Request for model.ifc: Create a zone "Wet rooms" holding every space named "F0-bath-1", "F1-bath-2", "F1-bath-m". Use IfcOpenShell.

First a look at what the model holds.

```python
import ifcopenshell

model = ifcopenshell.open("model.ifc")
print(model.schema)
seen = {}
for space in model.by_type("IfcSpace"):
    seen[space.LongName] = seen.get(space.LongName, 0) + 1
for name, count in sorted(seen.items(), key=str):
    print(count, "x", name)
print("zones:", [z.Name for z in model.by_type("IfcZone")][:20])
```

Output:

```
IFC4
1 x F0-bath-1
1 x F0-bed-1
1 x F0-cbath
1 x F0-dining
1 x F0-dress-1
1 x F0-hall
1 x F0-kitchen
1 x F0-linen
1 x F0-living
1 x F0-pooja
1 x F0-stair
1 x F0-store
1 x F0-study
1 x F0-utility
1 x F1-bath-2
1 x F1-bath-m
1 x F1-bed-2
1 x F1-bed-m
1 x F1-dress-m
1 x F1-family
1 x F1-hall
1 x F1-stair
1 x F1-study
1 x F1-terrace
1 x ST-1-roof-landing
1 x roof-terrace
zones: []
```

```python
import ifcopenshell
import ifcopenshell.api.group
import ifcopenshell.api.root

model = ifcopenshell.open("model.ifc")

names = {"F0-bath-1", "F1-bath-2", "F1-bath-m"}
spaces = [s for s in model.by_type("IfcSpace") if s.LongName in names]

zone = ifcopenshell.api.root.create_entity(model, ifc_class="IfcZone", name="Wet rooms")
ifcopenshell.api.group.assign_group(model, products=spaces, group=zone)
print(len(spaces), "spaces in", zone.Name)

model.write("model_rev.ifc")
```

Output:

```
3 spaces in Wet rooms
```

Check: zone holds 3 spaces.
